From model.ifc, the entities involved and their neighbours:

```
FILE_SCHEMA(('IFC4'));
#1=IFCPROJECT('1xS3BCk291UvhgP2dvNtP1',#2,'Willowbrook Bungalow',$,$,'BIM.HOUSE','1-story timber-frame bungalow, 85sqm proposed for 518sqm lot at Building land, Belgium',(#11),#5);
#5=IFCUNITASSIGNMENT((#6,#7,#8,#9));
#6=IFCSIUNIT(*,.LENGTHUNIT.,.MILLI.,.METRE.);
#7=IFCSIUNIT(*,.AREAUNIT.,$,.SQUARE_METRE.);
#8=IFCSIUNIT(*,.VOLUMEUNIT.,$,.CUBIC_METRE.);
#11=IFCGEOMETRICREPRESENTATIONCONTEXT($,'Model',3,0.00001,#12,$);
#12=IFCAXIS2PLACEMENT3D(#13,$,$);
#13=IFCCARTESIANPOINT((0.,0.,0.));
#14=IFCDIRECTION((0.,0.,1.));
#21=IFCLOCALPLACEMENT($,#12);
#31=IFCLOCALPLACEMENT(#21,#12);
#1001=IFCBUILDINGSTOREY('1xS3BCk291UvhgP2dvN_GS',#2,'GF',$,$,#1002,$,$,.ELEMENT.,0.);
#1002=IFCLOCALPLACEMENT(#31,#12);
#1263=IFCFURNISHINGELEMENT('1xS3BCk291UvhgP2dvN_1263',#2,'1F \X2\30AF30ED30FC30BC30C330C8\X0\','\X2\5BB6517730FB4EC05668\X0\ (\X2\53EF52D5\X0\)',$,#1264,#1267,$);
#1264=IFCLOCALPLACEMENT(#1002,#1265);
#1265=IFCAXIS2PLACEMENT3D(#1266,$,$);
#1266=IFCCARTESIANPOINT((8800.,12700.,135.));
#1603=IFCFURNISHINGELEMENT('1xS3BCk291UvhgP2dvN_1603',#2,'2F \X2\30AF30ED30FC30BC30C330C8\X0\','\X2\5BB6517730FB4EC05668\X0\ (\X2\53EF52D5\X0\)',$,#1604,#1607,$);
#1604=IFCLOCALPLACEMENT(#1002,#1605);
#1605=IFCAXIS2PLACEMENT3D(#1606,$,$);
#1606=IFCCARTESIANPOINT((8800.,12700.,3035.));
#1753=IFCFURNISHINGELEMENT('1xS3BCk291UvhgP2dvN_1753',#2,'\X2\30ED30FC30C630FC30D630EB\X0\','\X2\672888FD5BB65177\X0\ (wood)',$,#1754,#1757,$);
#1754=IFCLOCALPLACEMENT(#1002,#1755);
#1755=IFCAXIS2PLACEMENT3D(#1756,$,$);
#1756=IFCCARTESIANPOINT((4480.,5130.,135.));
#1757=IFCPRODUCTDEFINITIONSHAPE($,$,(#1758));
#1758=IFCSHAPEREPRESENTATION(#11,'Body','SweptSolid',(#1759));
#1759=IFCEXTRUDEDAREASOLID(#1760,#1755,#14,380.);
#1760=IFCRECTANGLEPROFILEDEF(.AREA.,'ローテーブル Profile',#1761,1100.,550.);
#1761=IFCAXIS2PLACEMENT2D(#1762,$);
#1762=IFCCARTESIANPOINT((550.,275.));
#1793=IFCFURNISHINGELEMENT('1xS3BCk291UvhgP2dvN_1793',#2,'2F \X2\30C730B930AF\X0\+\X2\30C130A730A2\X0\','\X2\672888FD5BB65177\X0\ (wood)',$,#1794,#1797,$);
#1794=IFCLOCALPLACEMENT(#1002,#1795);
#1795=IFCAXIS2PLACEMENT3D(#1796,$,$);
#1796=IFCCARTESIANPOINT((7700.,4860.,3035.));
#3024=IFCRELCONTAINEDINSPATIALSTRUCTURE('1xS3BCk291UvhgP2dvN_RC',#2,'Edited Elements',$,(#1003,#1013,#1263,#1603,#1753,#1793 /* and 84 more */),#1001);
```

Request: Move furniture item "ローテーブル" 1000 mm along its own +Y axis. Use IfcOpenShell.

```python
import ifcopenshell
import ifcopenshell.api.geometry
import ifcopenshell.util.placement
import ifcopenshell.util.unit

model = ifcopenshell.open("model.ifc")
unit_scale = ifcopenshell.util.unit.calculate_unit_scale(model)

item = model.by_guid("1xS3BCk291UvhgP2dvN_1753")
matrix = ifcopenshell.util.placement.get_local_placement(item.ObjectPlacement)
matrix[:3, 3] += matrix[:3, 1] * 1 / unit_scale
ifcopenshell.api.geometry.edit_object_placement(model, product=item, matrix=matrix, is_si=False)

print(ifcopenshell.util.placement.get_local_placement(item.ObjectPlacement).round(3) + 0.0)

model.write("model_updated.ifc")
```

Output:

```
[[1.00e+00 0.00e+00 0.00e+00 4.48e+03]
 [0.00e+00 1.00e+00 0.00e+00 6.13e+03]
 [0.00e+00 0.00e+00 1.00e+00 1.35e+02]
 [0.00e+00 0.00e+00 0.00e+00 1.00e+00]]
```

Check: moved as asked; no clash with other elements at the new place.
